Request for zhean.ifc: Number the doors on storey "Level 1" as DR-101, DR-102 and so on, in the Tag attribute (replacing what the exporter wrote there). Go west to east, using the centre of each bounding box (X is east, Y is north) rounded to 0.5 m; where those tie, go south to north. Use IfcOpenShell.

First a look at what the model holds.

```python
import ifcopenshell
import ifcopenshell.util.element
import ifcopenshell.util.placement

model = ifcopenshell.open("zhean.ifc")
print(model.schema)
storey = next(s for s in model.by_type("IfcBuildingStorey") if s.Name == "Level 1")
doors = [e for e in ifcopenshell.util.element.get_decomposition(storey) if e.is_a("IfcDoor")]
for e in sorted(doors, key=lambda e: e.id()):
    origin = ifcopenshell.util.placement.get_local_placement(e.ObjectPlacement)[:3, 3]
    print(e.id(), e.Tag, e.Name, origin.round(2) + 0.0, sep=" | ")
```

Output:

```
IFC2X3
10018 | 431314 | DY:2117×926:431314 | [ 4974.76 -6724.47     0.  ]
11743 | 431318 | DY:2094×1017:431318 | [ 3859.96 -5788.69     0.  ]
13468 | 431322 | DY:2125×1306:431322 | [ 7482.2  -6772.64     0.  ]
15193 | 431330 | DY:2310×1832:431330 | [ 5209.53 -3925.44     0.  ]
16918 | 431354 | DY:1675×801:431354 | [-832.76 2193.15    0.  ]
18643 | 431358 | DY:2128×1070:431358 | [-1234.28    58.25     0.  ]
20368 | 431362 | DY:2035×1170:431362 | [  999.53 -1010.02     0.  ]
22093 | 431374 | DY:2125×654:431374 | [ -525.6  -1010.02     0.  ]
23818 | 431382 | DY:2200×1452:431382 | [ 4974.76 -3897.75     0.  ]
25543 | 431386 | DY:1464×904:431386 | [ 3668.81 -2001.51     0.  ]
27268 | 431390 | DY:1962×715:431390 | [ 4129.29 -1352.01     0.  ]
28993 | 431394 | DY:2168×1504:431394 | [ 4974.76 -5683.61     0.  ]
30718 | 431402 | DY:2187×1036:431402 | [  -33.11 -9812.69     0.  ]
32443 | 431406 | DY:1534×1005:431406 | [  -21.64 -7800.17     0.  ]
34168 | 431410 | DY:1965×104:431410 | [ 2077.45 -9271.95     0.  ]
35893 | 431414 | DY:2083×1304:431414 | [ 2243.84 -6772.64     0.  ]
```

```python
import ifcopenshell
import ifcopenshell.geom
import ifcopenshell.util.element
import ifcopenshell.util.shape

model = ifcopenshell.open("zhean.ifc")
settings = ifcopenshell.geom.settings()
settings.set("use-world-coords", True)


def centre(element):
    shape = ifcopenshell.geom.create_shape(settings, element)
    return ifcopenshell.util.shape.get_bbox_centroid(shape.geometry)


storey = next(s for s in model.by_type("IfcBuildingStorey") if s.Name == "Level 1")
doors = [e for e in ifcopenshell.util.element.get_decomposition(storey) if e.is_a("IfcDoor")]

# Insertion points can sit at a corner or the storey origin, so sort by the geometry (in metres).
centres = {e: centre(e) for e in doors}
doors.sort(key=lambda e: (round(centres[e][0] / 0.5), centres[e][1]))

for i, e in enumerate(doors, start=1):
    number = f"DR-1{i:02d}"
    e.Tag = number
    print(e.id(), number)

model.write("zhean-out.ifc")
```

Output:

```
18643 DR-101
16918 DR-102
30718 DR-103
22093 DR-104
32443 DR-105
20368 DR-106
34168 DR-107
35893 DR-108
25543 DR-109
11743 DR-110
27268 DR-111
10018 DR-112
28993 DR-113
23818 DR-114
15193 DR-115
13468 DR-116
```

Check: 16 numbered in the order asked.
